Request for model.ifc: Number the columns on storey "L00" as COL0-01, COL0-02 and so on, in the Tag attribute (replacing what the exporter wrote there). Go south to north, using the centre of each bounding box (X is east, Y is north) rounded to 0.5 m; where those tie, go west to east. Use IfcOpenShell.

First a look at what the model holds.

```python
import ifcopenshell
import ifcopenshell.util.element
import ifcopenshell.util.placement

model = ifcopenshell.open("model.ifc")
print(model.schema)
storey = next(s for s in model.by_type("IfcBuildingStorey") if s.Name == "L00")
columns = [e for e in ifcopenshell.util.element.get_decomposition(storey) if e.is_a("IfcColumn")]
for e in sorted(columns, key=lambda e: e.id()):
    origin = ifcopenshell.util.placement.get_local_placement(e.ObjectPlacement)[:3, 3]
    print(e.id(), e.Tag, e.Name, origin.round(2) + 0.0, sep=" | ")
```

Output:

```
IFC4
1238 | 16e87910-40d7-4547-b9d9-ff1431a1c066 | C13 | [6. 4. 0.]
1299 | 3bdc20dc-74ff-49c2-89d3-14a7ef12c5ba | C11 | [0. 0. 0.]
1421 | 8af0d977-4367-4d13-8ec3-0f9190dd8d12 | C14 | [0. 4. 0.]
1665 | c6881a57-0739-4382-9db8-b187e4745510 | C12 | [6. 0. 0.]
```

```python
import ifcopenshell
import ifcopenshell.geom
import ifcopenshell.util.element
import ifcopenshell.util.shape

model = ifcopenshell.open("model.ifc")
settings = ifcopenshell.geom.settings()
settings.set("use-world-coords", True)


def centre(element):
    shape = ifcopenshell.geom.create_shape(settings, element)
    return ifcopenshell.util.shape.get_bbox_centroid(shape.geometry)


storey = next(s for s in model.by_type("IfcBuildingStorey") if s.Name == "L00")
columns = [e for e in ifcopenshell.util.element.get_decomposition(storey) if e.is_a("IfcColumn")]

# Insertion points can sit at a corner or the storey origin, so sort by the geometry (in metres).
centres = {e: centre(e) for e in columns}
columns.sort(key=lambda e: (round(centres[e][1] / 0.5), centres[e][0]))

for i, e in enumerate(columns, start=1):
    number = f"COL0-{i:02d}"
    e.Tag = number
    print(e.id(), number)

model.write("model-out.ifc")
```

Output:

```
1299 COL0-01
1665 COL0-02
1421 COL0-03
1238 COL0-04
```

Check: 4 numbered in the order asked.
